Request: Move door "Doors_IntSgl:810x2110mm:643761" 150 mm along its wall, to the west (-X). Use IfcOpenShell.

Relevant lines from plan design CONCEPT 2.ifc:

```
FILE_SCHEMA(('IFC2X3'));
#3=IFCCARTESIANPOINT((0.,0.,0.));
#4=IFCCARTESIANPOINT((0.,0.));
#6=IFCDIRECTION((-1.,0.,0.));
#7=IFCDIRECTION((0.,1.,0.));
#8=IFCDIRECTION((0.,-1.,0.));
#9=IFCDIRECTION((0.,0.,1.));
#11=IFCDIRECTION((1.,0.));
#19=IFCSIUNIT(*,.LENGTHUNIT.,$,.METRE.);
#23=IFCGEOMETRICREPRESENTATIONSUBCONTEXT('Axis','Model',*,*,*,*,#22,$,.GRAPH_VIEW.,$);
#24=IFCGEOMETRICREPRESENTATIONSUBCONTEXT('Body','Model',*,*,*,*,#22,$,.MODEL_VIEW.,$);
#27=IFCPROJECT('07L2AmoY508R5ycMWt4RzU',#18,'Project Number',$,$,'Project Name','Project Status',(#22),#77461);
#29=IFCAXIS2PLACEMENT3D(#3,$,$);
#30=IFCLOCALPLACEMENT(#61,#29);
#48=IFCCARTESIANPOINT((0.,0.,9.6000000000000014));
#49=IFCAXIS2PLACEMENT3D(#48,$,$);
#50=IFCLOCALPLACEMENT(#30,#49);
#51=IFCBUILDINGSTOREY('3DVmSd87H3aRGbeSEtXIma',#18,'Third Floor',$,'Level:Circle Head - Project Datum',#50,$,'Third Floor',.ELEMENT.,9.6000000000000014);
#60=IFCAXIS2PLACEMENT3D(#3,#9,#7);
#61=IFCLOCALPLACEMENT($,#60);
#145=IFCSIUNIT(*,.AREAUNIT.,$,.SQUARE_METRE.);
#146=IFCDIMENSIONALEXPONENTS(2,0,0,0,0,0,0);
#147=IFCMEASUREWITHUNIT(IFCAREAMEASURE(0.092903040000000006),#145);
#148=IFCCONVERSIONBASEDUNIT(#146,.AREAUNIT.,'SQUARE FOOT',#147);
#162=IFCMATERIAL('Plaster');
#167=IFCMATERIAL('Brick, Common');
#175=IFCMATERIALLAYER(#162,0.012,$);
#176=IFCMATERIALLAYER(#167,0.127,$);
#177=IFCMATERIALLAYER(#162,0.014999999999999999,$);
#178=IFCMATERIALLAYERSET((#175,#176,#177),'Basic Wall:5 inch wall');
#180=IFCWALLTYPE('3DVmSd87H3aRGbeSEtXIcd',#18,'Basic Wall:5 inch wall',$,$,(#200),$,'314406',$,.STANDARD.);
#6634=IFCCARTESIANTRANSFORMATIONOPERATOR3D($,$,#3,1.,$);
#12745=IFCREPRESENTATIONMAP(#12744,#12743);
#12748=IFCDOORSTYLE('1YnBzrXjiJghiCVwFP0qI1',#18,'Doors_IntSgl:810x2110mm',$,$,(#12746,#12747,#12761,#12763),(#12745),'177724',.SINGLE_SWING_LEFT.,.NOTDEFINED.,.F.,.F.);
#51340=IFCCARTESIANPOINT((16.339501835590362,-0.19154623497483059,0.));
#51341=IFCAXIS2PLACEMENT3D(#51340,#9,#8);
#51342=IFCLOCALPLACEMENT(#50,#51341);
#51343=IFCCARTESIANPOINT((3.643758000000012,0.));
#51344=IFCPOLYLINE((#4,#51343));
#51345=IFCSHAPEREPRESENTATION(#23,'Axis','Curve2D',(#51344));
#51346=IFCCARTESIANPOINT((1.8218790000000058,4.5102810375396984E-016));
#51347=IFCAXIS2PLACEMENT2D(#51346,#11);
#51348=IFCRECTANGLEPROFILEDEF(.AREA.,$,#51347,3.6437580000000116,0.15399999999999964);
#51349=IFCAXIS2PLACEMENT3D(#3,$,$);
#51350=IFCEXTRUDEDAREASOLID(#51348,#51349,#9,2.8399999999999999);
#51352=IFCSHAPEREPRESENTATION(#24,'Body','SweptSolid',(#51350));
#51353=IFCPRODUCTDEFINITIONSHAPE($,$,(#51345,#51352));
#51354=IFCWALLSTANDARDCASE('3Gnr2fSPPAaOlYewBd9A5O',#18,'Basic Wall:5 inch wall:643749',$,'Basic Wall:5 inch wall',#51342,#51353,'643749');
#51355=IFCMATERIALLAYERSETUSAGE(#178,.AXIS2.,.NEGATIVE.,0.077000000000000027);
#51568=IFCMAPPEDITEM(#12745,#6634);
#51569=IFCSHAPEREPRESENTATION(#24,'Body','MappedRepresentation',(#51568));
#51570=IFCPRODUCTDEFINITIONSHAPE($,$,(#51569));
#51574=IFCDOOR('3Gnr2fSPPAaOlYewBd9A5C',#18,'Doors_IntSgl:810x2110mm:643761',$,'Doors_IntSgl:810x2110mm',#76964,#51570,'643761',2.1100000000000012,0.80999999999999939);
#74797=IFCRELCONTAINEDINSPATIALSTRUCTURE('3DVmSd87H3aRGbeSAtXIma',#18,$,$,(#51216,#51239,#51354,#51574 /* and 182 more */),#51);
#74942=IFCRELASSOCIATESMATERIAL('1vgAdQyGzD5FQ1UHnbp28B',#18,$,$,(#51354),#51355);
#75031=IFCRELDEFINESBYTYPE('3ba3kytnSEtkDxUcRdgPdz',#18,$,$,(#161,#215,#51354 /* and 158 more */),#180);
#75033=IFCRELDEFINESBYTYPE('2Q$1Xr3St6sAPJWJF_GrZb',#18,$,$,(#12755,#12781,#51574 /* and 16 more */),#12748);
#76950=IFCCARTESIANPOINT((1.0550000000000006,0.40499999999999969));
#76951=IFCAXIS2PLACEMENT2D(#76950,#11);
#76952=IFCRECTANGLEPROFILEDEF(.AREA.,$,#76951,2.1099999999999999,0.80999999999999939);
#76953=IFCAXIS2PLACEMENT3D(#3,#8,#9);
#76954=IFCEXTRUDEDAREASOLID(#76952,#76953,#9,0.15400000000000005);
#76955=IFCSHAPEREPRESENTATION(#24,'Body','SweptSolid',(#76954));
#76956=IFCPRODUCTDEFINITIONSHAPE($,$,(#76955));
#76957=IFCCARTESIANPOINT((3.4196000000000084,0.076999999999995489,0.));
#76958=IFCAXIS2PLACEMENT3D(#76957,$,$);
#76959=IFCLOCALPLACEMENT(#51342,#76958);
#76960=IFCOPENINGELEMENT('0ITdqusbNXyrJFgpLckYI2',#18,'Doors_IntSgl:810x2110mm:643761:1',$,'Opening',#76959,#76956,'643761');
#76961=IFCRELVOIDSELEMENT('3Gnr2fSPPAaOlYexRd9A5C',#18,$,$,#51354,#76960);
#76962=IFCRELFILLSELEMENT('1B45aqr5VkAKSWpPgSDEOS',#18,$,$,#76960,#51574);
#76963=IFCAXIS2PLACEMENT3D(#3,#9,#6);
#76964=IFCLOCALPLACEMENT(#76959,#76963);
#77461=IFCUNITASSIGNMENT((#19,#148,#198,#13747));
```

```python
import ifcopenshell
import ifcopenshell.api.geometry
import ifcopenshell.util.placement
import ifcopenshell.util.unit

model = ifcopenshell.open("plan design CONCEPT 2.ifc")
unit_scale = ifcopenshell.util.unit.calculate_unit_scale(model)

door = model.by_guid("3Gnr2fSPPAaOlYewBd9A5C")
opening = door.FillsVoids[0].RelatingOpeningElement
wall = opening.VoidsElements[0].RelatingBuildingElement

wall_matrix = ifcopenshell.util.placement.get_local_placement(wall.ObjectPlacement)
shift = wall_matrix[:3, 0] * -0.15 / unit_scale
before = ifcopenshell.util.placement.get_local_placement(door.ObjectPlacement)[:3, 3].copy()

# The door is placed relative to its opening, so it follows when the opening moves.
matrix = ifcopenshell.util.placement.get_local_placement(opening.ObjectPlacement)
matrix[:3, 3] += shift
ifcopenshell.api.geometry.edit_object_placement(
    model, product=opening, matrix=matrix, is_si=False, should_transform_children=True
)

after = ifcopenshell.util.placement.get_local_placement(door.ObjectPlacement)[:3, 3]
print("door moved by", (after - before).round(3) + 0.0)

model.write("plan design CONCEPT 2_edited.ifc")
```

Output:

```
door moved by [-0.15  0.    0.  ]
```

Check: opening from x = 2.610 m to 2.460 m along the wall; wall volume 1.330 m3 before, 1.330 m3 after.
